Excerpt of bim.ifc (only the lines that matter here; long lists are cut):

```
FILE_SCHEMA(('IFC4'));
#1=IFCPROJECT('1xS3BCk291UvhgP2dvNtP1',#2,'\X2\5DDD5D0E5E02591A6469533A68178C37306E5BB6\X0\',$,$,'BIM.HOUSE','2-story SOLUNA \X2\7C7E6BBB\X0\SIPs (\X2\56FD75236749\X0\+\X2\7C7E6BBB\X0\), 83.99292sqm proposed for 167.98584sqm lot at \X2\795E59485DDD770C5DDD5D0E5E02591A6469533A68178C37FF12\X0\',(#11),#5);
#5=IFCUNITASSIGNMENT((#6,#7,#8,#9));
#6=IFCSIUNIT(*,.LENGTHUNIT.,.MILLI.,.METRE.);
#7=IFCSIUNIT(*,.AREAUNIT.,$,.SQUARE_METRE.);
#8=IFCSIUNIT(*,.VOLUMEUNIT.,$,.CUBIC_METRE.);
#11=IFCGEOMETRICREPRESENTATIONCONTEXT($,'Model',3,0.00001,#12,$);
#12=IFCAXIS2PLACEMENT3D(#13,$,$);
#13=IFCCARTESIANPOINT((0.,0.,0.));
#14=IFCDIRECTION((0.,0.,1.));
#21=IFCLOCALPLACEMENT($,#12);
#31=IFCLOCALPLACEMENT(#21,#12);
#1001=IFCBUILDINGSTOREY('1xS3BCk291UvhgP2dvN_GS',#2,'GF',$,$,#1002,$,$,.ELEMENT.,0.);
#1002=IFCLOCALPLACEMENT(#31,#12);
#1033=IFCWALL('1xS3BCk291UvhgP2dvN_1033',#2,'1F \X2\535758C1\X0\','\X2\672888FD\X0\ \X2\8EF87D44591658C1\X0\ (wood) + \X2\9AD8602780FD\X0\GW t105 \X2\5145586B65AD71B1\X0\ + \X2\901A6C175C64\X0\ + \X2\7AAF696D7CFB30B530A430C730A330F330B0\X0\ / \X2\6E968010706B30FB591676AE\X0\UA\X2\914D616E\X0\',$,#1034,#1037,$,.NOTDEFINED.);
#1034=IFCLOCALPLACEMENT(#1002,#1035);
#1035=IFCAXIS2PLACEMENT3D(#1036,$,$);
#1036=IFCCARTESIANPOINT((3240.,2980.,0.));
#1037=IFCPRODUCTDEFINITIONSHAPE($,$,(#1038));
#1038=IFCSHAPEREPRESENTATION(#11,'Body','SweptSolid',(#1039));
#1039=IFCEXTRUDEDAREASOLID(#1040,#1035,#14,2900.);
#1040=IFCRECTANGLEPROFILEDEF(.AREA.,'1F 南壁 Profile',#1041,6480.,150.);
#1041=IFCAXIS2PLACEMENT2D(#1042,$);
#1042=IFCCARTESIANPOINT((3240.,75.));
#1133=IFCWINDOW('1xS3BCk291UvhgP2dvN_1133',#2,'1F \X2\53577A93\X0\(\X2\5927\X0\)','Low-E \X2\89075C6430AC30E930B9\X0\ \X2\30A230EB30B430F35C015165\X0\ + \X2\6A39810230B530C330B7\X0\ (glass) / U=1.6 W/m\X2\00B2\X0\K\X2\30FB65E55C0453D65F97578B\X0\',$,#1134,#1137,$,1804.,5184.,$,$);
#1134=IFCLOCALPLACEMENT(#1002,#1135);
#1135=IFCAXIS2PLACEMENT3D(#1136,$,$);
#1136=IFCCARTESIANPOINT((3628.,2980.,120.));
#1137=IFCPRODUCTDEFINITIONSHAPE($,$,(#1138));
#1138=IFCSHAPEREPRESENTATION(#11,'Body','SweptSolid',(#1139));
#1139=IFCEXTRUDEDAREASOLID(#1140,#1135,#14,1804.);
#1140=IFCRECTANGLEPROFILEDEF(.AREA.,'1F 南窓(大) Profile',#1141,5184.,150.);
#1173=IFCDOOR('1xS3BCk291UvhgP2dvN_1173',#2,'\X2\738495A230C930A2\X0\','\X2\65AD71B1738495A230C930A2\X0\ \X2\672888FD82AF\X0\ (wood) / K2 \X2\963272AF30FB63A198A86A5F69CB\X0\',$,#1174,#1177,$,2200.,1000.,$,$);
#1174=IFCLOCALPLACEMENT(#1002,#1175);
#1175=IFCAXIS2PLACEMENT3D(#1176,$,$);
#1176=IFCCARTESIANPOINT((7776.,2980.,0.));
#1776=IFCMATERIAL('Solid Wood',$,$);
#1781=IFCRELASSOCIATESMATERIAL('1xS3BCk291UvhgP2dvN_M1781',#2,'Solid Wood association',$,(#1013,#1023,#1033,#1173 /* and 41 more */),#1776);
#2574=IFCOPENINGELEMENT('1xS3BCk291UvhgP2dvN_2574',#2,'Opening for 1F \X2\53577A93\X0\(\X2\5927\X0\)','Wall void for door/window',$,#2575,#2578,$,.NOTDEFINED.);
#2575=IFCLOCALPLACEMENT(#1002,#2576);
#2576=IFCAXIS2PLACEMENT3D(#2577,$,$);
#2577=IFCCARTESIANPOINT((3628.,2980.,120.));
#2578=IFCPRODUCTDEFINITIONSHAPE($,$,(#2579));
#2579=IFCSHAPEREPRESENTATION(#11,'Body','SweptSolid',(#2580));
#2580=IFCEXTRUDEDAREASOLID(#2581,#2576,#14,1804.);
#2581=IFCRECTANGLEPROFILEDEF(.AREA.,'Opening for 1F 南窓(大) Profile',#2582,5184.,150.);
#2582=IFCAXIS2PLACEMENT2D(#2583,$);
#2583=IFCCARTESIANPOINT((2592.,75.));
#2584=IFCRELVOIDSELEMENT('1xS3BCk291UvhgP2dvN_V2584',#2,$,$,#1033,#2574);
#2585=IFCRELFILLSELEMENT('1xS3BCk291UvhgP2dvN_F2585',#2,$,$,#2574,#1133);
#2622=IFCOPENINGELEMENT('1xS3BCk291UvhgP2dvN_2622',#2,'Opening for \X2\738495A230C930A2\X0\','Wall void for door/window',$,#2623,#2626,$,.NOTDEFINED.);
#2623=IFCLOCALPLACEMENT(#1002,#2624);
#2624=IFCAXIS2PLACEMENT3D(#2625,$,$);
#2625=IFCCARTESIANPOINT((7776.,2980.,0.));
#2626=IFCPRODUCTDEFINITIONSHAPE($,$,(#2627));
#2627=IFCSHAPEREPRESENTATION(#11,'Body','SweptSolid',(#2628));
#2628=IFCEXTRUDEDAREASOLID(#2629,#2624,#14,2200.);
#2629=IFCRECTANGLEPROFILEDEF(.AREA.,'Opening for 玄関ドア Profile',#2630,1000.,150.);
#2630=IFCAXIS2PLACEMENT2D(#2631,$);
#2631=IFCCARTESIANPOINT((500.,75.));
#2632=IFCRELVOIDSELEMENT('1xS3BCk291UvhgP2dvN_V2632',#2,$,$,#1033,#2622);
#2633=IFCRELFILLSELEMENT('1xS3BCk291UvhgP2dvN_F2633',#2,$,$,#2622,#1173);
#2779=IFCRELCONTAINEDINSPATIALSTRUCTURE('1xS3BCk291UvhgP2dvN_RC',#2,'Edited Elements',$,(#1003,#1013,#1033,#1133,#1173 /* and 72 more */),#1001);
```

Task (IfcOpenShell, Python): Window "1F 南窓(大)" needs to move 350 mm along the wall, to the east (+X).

```python
import ifcopenshell
import ifcopenshell.api.geometry
import ifcopenshell.util.placement
import ifcopenshell.util.unit

model = ifcopenshell.open("bim.ifc")
unit_scale = ifcopenshell.util.unit.calculate_unit_scale(model)

window = model.by_id(1133)
opening = window.FillsVoids[0].RelatingOpeningElement
wall = opening.VoidsElements[0].RelatingBuildingElement

wall_matrix = ifcopenshell.util.placement.get_local_placement(wall.ObjectPlacement)
shift = wall_matrix[:3, 0] * 0.35 / unit_scale
before = ifcopenshell.util.placement.get_local_placement(window.ObjectPlacement)[:3, 3].copy()

# The window is not placed relative to its opening, so move both.
for product in (opening, window):
    matrix = ifcopenshell.util.placement.get_local_placement(product.ObjectPlacement)
    matrix[:3, 3] += shift
    ifcopenshell.api.geometry.edit_object_placement(model, product=product, matrix=matrix, is_si=False)

after = ifcopenshell.util.placement.get_local_placement(window.ObjectPlacement)[:3, 3]
print("window moved by", (after - before).round(3) + 0.0)

model.write("bim-out.ifc")
```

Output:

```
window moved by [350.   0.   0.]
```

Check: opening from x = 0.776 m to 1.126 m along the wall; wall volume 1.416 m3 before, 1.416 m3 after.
